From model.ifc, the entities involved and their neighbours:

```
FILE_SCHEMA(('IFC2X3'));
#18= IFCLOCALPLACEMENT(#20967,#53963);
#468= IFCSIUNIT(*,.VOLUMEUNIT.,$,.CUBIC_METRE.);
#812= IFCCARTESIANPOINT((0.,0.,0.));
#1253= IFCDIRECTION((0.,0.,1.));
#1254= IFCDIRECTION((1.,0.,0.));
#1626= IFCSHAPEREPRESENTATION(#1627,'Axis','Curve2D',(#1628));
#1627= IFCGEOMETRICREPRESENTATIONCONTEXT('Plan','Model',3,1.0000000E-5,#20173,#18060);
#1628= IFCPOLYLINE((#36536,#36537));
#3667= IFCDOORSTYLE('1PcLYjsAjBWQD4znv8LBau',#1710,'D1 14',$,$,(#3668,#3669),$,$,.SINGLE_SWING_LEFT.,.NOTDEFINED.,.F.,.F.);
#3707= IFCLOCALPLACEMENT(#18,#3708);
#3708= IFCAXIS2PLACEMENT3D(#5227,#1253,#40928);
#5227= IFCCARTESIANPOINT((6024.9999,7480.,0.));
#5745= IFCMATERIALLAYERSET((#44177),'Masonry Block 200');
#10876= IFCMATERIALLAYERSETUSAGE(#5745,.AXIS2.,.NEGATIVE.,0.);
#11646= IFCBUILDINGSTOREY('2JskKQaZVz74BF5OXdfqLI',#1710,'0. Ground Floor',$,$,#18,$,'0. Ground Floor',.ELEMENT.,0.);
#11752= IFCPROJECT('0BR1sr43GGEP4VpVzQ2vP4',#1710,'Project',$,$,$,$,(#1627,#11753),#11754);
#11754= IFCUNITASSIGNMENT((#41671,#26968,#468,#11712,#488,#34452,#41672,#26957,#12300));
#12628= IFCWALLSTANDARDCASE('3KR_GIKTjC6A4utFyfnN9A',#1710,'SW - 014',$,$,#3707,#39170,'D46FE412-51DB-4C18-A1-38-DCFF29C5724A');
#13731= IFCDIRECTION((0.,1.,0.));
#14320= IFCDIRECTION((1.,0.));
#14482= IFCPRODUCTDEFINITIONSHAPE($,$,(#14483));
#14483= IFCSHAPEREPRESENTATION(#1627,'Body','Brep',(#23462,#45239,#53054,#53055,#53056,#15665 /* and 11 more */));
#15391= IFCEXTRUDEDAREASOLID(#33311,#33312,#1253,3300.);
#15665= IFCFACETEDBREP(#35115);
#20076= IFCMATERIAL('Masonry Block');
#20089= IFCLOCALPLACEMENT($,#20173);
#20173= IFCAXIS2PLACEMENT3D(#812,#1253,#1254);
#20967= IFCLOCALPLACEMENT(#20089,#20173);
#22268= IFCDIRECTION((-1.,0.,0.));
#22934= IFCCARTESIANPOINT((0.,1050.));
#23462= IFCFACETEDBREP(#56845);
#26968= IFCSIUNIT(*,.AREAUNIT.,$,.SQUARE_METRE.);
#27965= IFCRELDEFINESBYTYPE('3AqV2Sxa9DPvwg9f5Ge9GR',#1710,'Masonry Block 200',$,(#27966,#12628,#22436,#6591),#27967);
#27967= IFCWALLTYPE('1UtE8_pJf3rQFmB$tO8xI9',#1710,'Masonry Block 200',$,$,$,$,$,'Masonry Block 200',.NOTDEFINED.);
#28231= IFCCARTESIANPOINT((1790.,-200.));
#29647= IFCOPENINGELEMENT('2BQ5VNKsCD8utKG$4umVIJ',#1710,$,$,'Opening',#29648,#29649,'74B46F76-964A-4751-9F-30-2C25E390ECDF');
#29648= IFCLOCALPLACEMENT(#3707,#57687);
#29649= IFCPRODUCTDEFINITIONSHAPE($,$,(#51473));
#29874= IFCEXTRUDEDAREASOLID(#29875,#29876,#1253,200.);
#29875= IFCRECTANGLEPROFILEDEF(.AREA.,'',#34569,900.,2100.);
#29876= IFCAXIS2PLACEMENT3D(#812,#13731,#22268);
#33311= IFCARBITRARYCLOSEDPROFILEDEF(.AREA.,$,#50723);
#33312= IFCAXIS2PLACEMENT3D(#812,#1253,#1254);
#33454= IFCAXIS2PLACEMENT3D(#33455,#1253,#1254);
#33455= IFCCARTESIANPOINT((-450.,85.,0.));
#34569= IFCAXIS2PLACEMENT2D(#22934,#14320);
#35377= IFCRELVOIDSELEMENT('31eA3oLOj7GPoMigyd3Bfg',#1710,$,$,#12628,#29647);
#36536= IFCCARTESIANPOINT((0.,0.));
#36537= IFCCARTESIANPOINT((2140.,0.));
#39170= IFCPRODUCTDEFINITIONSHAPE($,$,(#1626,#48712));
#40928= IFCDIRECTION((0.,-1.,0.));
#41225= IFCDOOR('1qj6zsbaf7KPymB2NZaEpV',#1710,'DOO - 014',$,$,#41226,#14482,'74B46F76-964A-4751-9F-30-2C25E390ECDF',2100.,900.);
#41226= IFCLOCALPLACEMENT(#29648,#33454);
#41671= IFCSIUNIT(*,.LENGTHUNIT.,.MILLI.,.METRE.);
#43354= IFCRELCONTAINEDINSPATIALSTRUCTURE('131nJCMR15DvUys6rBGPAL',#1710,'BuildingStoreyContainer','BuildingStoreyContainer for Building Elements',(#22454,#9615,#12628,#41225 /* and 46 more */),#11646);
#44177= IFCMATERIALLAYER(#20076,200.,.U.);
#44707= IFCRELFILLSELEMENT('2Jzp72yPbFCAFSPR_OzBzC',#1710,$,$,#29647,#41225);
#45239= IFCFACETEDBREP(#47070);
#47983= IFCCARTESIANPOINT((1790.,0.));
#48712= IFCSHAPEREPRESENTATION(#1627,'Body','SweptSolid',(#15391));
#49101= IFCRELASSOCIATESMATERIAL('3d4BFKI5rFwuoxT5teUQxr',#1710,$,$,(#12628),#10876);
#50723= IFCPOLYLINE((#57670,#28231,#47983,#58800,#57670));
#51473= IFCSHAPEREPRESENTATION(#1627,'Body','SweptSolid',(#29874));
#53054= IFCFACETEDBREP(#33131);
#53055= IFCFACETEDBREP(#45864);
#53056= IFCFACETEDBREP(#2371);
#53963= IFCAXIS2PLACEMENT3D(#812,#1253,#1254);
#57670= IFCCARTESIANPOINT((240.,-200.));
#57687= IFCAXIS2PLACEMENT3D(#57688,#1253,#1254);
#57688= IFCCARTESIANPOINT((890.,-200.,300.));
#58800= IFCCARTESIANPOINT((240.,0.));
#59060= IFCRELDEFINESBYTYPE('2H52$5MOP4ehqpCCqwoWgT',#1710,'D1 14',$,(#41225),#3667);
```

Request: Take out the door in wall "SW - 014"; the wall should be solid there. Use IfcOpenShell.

```python
import ifcopenshell
import ifcopenshell.api.feature
import ifcopenshell.api.root
import ifcopenshell.geom
import ifcopenshell.util.shape

model = ifcopenshell.open("model.ifc")
settings = ifcopenshell.geom.settings()


def volume(element):
    """Net volume in cubic metres, openings subtracted."""
    shape = ifcopenshell.geom.create_shape(settings, element)
    return ifcopenshell.util.shape.get_volume(shape.geometry)


door = model.by_guid("1qj6zsbaf7KPymB2NZaEpV")
opening = door.FillsVoids[0].RelatingOpeningElement
wall = opening.VoidsElements[0].RelatingBuildingElement
before = volume(wall)

ifcopenshell.api.root.remove_product(model, product=door)
ifcopenshell.api.feature.remove_feature(model, feature=opening)

after = volume(wall)

print(f"wall volume {before:.3f} -> {after:.3f} m3")

model.write("model_updated.ifc")
```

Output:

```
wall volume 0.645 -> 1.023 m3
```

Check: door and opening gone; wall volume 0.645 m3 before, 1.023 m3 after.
